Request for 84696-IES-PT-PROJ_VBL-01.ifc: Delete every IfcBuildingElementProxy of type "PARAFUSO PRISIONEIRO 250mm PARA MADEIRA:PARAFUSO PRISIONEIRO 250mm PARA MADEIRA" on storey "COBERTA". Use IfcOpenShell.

First a look at what the model holds.

```python
import ifcopenshell
import ifcopenshell.util.element

model = ifcopenshell.open("84696-IES-PT-PROJ_VBL-01.ifc")
print(model.schema)
storey = next(s for s in model.by_type("IfcBuildingStorey") if s.Name == "COBERTA")
proxies = [e for e in ifcopenshell.util.element.get_decomposition(storey) if e.is_a("IfcBuildingElementProxy")]
seen = {}
for e in proxies:
    element_type = ifcopenshell.util.element.get_type(e)
    name = element_type.Name if element_type not in (None, e) else None
    seen[name] = seen.get(name, 0) + 1
for name, count in sorted(seen.items(), key=str):
    print(count, "x", name)
```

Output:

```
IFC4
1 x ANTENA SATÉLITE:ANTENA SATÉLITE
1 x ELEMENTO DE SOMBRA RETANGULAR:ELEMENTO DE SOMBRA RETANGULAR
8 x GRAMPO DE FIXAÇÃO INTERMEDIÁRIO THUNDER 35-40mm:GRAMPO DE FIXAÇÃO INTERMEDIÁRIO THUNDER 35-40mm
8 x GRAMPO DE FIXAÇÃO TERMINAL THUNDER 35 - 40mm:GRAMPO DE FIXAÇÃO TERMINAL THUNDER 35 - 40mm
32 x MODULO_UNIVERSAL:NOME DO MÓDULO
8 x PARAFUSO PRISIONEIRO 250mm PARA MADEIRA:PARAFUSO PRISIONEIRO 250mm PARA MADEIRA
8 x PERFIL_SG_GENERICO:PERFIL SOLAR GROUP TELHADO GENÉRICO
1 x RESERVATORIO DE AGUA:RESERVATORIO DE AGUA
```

```python
import ifcopenshell
import ifcopenshell.api.root
import ifcopenshell.util.element

model = ifcopenshell.open("84696-IES-PT-PROJ_VBL-01.ifc")

storey = next(s for s in model.by_type("IfcBuildingStorey") if s.Name == "COBERTA")
proxies = [e for e in ifcopenshell.util.element.get_decomposition(storey) if e.is_a("IfcBuildingElementProxy")]
targets = [e for e in proxies if (t := ifcopenshell.util.element.get_type(e)) not in (None, e) and t.Name == "PARAFUSO PRISIONEIRO 250mm PARA MADEIRA:PARAFUSO PRISIONEIRO 250mm PARA MADEIRA"]

for e in targets:
    ifcopenshell.api.root.remove_product(model, product=e)
print(len(targets), "removed")

model.write("84696-IES-PT-PROJ_VBL-01-out.ifc")
```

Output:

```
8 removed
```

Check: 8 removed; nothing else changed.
